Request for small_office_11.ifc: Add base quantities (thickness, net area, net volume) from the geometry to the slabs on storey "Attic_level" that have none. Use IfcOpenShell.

First a look at what the model holds.

```python
import ifcopenshell
import ifcopenshell.util.element
import ifcopenshell.util.unit

model = ifcopenshell.open("small_office_11.ifc")
print(model.schema)
for unit_type in ("LENGTHUNIT", "AREAUNIT", "VOLUMEUNIT"):
    print(unit_type, ifcopenshell.util.unit.calculate_unit_scale(model, unit_type))
storey = next(s for s in model.by_type("IfcBuildingStorey") if s.Name == "Attic_level")
slabs = [e for e in ifcopenshell.util.element.get_decomposition(storey) if e.is_a("IfcSlab")]
for e in sorted(slabs, key=lambda e: e.id()):
    print(e.id(), e.is_a(), e.Name, list(ifcopenshell.util.element.get_psets(e, qtos_only=True)), sep=" | ")
```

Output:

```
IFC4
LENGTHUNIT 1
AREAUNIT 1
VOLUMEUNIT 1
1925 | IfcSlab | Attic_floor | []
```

```python
import ifcopenshell
import ifcopenshell.api.pset
import ifcopenshell.geom
import ifcopenshell.util.element
import ifcopenshell.util.shape
import ifcopenshell.util.unit

model = ifcopenshell.open("small_office_11.ifc")
unit_scale = ifcopenshell.util.unit.calculate_unit_scale(model)
area_scale = ifcopenshell.util.unit.calculate_unit_scale(model, "AREAUNIT")
volume_scale = ifcopenshell.util.unit.calculate_unit_scale(model, "VOLUMEUNIT")
settings = ifcopenshell.geom.settings()

storey = next(s for s in model.by_type("IfcBuildingStorey") if s.Name == "Attic_level")
slabs = [e for e in ifcopenshell.util.element.get_decomposition(storey) if e.is_a("IfcSlab")]

for e in sorted(slabs, key=lambda e: e.id()):
    if ifcopenshell.util.element.get_psets(e, qtos_only=True, should_inherit=False):
        continue
    # Geometry comes back in metres, in the element's own axes.
    shape = ifcopenshell.geom.create_shape(settings, e)
    values = {
        "Width": ifcopenshell.util.shape.get_z(shape.geometry) / unit_scale,
        "NetArea": ifcopenshell.util.shape.get_footprint_area(shape.geometry) / area_scale,
        "NetVolume": ifcopenshell.util.shape.get_volume(shape.geometry) / volume_scale,
    }
    qto = ifcopenshell.api.pset.add_qto(model, product=e, name="Qto_SlabBaseQuantities")
    ifcopenshell.api.pset.edit_qto(model, qto=qto, properties=values)
    print(e.id(), {k: round(v, 3) for k, v in values.items()})

model.write("small_office_11_rev.ifc")
```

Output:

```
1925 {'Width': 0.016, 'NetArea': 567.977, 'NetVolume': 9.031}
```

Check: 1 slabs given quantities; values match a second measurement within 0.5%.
